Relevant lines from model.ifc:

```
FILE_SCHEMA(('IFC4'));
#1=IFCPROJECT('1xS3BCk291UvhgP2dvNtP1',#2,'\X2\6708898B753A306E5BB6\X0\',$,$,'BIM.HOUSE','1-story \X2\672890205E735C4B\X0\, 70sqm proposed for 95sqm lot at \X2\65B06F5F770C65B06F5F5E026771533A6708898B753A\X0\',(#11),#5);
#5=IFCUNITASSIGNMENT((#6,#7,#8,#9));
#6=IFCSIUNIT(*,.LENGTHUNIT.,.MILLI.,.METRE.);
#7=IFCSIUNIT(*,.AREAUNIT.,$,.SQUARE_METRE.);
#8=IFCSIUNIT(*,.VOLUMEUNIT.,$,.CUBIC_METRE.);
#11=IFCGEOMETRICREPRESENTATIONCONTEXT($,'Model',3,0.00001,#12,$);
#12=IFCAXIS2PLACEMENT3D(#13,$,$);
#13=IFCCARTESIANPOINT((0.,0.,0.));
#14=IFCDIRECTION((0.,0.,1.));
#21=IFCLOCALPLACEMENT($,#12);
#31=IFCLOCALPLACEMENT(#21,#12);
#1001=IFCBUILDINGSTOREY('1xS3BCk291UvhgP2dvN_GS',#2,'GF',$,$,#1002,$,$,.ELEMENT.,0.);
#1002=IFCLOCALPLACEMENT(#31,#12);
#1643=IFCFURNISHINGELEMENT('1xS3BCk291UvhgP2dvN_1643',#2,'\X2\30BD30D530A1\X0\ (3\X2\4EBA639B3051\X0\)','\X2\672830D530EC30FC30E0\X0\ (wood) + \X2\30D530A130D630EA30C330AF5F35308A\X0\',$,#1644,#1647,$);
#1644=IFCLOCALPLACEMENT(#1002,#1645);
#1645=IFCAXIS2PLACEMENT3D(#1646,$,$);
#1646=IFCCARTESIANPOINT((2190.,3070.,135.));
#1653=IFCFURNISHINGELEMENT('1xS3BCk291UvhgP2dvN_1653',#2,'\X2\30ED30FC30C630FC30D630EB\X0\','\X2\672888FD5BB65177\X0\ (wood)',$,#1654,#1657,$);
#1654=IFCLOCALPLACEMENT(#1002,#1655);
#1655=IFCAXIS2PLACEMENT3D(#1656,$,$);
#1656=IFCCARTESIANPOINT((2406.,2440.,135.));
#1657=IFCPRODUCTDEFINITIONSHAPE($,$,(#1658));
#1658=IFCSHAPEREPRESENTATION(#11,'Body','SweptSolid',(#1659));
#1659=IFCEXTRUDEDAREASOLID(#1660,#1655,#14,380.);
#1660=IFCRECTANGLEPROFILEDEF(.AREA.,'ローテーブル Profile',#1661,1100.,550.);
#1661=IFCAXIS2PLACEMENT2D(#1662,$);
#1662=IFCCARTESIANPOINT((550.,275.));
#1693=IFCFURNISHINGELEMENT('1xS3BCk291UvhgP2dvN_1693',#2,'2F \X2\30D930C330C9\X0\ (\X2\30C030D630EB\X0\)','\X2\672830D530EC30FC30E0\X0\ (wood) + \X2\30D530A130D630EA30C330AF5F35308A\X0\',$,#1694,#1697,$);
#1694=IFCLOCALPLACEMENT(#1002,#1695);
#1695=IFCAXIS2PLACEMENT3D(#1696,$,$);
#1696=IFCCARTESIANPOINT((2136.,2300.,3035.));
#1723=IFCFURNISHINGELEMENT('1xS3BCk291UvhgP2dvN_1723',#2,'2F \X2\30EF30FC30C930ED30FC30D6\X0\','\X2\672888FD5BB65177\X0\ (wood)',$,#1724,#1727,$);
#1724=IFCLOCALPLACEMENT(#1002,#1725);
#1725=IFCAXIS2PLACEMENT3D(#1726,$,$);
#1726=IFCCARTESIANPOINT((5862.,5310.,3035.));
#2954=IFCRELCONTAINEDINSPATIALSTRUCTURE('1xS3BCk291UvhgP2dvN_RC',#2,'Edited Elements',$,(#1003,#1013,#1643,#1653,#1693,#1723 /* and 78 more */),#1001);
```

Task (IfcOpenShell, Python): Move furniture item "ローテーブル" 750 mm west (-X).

```python
import ifcopenshell
import ifcopenshell.api.geometry
import ifcopenshell.util.placement
import ifcopenshell.util.unit

model = ifcopenshell.open("model.ifc")
unit_scale = ifcopenshell.util.unit.calculate_unit_scale(model)

item = model.by_guid("1xS3BCk291UvhgP2dvN_1653")
matrix = ifcopenshell.util.placement.get_local_placement(item.ObjectPlacement)
matrix[0, 3] -= 0.75 / unit_scale
ifcopenshell.api.geometry.edit_object_placement(model, product=item, matrix=matrix, is_si=False)

print(ifcopenshell.util.placement.get_local_placement(item.ObjectPlacement).round(3) + 0.0)

model.write("model-out.ifc")
```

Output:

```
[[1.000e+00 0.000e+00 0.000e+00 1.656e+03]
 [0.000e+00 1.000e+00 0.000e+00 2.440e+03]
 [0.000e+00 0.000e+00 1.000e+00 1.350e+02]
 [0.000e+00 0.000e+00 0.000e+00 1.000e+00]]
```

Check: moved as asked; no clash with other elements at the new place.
